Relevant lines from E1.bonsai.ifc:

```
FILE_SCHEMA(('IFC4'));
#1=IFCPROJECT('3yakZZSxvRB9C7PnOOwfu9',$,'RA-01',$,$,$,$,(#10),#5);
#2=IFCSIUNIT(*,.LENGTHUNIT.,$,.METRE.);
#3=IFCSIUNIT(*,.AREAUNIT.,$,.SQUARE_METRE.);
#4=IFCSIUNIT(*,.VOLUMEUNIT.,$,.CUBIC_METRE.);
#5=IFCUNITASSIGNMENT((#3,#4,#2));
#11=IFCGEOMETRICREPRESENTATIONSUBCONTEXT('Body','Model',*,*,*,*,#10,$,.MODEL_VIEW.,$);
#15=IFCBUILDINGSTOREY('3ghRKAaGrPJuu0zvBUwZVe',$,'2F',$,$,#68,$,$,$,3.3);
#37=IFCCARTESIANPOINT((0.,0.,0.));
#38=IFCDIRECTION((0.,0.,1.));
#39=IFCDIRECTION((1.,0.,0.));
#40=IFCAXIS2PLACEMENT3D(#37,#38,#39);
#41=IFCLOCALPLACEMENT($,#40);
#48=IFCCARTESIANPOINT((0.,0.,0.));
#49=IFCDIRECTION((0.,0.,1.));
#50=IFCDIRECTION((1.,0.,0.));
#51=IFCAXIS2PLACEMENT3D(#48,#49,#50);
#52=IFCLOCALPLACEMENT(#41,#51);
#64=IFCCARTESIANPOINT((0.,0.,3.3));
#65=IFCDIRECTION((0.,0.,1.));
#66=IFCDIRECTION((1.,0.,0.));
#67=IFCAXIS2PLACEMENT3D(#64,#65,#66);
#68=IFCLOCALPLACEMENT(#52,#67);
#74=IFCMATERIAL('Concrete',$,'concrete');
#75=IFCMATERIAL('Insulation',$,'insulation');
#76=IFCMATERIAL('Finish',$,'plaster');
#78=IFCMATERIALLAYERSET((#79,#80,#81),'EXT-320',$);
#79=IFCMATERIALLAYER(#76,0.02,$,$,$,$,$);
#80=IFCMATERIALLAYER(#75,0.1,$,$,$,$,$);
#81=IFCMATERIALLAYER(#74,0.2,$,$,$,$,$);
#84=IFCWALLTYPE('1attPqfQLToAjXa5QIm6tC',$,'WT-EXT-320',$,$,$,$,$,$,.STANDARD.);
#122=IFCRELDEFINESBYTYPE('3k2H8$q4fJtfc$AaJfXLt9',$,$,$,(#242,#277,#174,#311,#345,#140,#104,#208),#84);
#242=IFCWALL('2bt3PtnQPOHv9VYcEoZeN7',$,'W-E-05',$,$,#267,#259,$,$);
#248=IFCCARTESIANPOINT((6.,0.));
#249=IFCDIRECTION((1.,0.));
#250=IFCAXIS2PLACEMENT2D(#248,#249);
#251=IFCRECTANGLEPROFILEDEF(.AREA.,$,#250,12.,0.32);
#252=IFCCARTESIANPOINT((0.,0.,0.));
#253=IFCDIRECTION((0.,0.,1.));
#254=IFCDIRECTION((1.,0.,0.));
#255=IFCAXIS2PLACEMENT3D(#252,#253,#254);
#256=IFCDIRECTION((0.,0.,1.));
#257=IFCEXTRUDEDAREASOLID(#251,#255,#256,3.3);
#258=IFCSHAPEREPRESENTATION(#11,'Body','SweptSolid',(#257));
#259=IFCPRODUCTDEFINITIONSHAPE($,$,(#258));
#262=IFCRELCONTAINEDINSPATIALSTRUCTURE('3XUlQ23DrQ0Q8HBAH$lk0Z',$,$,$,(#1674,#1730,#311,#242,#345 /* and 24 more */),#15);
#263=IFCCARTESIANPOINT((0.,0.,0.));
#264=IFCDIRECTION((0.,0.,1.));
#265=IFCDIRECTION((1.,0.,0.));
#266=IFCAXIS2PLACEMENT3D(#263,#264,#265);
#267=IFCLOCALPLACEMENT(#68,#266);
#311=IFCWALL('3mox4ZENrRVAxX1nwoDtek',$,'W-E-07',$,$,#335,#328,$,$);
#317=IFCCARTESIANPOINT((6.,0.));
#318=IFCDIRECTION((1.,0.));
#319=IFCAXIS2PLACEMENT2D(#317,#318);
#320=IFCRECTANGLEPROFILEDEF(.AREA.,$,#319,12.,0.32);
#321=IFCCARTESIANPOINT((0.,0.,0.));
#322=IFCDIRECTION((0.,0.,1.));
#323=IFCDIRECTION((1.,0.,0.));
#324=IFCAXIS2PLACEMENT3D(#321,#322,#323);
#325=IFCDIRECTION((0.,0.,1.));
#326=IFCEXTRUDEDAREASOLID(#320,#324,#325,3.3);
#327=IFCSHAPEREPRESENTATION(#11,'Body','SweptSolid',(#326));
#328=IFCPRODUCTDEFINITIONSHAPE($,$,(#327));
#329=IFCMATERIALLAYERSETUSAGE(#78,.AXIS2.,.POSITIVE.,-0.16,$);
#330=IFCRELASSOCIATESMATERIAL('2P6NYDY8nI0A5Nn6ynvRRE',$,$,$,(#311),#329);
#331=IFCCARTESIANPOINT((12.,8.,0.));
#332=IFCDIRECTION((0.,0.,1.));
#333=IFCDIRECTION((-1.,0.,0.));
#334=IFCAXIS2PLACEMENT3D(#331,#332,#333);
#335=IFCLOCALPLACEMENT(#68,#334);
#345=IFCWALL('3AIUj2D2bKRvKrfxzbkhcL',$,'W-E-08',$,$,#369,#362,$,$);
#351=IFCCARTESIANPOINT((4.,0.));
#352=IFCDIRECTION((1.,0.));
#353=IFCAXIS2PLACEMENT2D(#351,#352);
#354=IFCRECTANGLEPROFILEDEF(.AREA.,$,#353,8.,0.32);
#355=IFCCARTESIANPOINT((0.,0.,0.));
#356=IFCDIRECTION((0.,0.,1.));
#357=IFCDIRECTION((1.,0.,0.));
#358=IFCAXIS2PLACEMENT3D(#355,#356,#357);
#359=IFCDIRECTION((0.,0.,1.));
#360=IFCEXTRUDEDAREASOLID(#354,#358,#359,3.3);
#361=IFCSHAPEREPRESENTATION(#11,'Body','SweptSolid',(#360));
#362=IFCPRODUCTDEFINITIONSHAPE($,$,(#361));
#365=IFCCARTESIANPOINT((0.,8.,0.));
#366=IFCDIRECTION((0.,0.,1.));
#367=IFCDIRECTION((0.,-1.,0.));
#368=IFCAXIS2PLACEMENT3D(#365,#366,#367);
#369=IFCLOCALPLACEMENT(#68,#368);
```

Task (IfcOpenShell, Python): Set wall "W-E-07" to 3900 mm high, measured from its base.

```python
import ifcopenshell
import ifcopenshell.geom
import ifcopenshell.util.representation
import ifcopenshell.util.shape

model = ifcopenshell.open("E1.bonsai.ifc")
settings = ifcopenshell.geom.settings()


def volume(element):
    """Net volume in cubic metres, openings subtracted."""
    shape = ifcopenshell.geom.create_shape(settings, element)
    return ifcopenshell.util.shape.get_volume(shape.geometry)


wall = model.by_id(311)
before = volume(wall)

body = ifcopenshell.util.representation.get_representation(wall, "Model", "Body")
solid = body.Items[0]
old_height = solid.Depth
solid.Depth = 3.9
after = volume(wall)

print(f"height {old_height:g} -> {solid.Depth:g}, volume {before:.3f} -> {after:.3f} m3")

model.write("E1.bonsai_v2.ifc")
```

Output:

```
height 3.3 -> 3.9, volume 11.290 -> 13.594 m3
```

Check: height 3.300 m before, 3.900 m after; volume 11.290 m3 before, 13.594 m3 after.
